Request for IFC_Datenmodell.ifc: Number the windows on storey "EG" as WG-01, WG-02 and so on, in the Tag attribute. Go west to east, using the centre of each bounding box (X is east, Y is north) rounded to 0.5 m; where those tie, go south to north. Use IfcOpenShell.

First a look at what the model holds.

```python
import ifcopenshell
import ifcopenshell.util.element
import ifcopenshell.util.placement

model = ifcopenshell.open("IFC_Datenmodell.ifc")
print(model.schema)
storey = next(s for s in model.by_type("IfcBuildingStorey") if s.Name == "EG")
windows = [e for e in ifcopenshell.util.element.get_decomposition(storey) if e.is_a("IfcWindow")]
for e in sorted(windows, key=lambda e: e.id()):
    origin = ifcopenshell.util.placement.get_local_placement(e.ObjectPlacement)[:3, 3]
    print(e.id(), e.Tag, e.Name, origin.round(2) + 0.0, sep=" | ")
```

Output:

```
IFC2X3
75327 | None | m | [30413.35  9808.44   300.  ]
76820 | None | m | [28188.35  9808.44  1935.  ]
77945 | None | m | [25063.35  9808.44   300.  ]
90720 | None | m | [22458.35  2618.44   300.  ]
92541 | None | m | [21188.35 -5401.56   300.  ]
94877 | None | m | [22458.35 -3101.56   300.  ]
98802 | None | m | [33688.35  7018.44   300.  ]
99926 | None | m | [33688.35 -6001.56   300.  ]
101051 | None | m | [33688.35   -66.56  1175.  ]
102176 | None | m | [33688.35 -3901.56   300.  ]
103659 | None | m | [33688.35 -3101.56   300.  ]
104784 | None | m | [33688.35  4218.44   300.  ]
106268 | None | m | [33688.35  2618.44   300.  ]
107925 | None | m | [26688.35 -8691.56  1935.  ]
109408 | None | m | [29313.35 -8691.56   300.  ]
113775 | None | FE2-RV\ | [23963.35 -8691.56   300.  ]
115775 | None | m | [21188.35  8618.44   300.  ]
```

```python
import ifcopenshell
import ifcopenshell.geom
import ifcopenshell.util.element
import ifcopenshell.util.shape

model = ifcopenshell.open("IFC_Datenmodell.ifc")
settings = ifcopenshell.geom.settings()
settings.set("use-world-coords", True)


def centre(element):
    shape = ifcopenshell.geom.create_shape(settings, element)
    return ifcopenshell.util.shape.get_bbox_centroid(shape.geometry)


storey = next(s for s in model.by_type("IfcBuildingStorey") if s.Name == "EG")
windows = [e for e in ifcopenshell.util.element.get_decomposition(storey) if e.is_a("IfcWindow")]

# Insertion points can sit at a corner or the storey origin, so sort by the geometry (in metres).
centres = {e: centre(e) for e in windows}
windows.sort(key=lambda e: (round(centres[e][0] / 0.5), centres[e][1]))

for i, e in enumerate(windows, start=1):
    number = f"WG-{i:02d}"
    e.Tag = number
    print(e.id(), number)

model.write("IFC_Datenmodell_rev.ifc")
```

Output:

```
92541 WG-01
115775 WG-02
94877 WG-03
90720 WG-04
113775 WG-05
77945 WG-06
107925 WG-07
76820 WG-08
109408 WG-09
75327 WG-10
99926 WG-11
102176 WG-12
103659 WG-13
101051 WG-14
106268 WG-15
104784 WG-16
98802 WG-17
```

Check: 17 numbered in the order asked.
